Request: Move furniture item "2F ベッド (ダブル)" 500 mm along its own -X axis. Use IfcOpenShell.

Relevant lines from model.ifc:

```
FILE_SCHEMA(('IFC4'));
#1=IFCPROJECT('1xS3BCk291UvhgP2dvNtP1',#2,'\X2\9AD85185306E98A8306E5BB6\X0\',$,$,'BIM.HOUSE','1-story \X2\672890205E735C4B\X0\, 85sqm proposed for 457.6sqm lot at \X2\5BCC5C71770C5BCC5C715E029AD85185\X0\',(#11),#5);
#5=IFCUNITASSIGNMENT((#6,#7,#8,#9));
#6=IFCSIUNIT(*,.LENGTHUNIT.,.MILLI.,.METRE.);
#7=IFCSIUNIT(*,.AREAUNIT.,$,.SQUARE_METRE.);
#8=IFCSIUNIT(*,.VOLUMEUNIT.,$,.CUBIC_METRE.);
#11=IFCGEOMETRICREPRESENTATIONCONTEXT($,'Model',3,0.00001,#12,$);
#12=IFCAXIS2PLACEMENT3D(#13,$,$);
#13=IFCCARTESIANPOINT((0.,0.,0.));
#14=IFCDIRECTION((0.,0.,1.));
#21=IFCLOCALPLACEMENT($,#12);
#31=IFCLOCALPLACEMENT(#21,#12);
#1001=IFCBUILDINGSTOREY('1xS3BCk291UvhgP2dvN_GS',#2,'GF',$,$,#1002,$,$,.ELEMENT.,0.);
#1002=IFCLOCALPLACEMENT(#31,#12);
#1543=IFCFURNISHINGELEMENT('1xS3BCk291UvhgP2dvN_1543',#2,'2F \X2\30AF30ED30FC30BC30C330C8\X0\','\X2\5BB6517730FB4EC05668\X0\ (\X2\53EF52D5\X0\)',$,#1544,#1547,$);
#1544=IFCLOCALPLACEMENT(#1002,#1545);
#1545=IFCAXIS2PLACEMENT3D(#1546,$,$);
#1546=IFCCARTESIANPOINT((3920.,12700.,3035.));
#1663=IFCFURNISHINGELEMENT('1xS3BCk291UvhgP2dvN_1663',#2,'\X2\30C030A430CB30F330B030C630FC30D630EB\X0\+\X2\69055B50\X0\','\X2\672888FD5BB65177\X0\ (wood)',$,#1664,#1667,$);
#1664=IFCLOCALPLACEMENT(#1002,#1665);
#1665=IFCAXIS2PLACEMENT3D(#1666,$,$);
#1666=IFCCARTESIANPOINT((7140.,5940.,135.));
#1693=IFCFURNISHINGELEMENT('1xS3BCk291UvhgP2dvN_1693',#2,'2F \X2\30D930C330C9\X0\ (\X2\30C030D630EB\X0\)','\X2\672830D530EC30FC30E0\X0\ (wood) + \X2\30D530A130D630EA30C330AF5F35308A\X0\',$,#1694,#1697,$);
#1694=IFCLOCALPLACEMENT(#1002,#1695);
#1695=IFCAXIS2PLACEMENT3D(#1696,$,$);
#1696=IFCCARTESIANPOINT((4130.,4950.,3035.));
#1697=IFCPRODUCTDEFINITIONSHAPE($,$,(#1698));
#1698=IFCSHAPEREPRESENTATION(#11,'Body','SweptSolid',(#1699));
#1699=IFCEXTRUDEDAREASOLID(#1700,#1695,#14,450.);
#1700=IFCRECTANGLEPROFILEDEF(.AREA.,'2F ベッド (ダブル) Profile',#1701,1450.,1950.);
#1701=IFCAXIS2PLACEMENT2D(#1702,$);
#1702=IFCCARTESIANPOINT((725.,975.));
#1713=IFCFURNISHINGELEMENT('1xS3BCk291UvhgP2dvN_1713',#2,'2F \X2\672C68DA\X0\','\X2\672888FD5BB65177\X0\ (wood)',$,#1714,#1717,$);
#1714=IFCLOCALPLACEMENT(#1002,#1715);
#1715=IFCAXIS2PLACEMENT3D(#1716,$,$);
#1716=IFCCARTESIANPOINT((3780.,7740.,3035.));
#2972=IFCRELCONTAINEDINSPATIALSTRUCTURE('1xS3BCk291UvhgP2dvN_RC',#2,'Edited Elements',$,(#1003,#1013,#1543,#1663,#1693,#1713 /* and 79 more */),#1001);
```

```python
import ifcopenshell
import ifcopenshell.api.geometry
import ifcopenshell.util.placement

model = ifcopenshell.open("model.ifc")

item = model.by_guid("1xS3BCk291UvhgP2dvN_1693")
matrix = ifcopenshell.util.placement.get_local_placement(item.ObjectPlacement)
matrix[:3, 3] -= matrix[:3, 0] * 500.0
ifcopenshell.api.geometry.edit_object_placement(model, product=item, matrix=matrix, is_si=False)

print(ifcopenshell.util.placement.get_local_placement(item.ObjectPlacement).round(3) + 0.0)

model.write("model_v2.ifc")
```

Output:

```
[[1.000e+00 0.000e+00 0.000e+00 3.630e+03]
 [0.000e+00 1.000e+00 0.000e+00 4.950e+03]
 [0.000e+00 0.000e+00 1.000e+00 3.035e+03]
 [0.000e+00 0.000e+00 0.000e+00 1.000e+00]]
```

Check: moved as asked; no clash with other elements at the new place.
